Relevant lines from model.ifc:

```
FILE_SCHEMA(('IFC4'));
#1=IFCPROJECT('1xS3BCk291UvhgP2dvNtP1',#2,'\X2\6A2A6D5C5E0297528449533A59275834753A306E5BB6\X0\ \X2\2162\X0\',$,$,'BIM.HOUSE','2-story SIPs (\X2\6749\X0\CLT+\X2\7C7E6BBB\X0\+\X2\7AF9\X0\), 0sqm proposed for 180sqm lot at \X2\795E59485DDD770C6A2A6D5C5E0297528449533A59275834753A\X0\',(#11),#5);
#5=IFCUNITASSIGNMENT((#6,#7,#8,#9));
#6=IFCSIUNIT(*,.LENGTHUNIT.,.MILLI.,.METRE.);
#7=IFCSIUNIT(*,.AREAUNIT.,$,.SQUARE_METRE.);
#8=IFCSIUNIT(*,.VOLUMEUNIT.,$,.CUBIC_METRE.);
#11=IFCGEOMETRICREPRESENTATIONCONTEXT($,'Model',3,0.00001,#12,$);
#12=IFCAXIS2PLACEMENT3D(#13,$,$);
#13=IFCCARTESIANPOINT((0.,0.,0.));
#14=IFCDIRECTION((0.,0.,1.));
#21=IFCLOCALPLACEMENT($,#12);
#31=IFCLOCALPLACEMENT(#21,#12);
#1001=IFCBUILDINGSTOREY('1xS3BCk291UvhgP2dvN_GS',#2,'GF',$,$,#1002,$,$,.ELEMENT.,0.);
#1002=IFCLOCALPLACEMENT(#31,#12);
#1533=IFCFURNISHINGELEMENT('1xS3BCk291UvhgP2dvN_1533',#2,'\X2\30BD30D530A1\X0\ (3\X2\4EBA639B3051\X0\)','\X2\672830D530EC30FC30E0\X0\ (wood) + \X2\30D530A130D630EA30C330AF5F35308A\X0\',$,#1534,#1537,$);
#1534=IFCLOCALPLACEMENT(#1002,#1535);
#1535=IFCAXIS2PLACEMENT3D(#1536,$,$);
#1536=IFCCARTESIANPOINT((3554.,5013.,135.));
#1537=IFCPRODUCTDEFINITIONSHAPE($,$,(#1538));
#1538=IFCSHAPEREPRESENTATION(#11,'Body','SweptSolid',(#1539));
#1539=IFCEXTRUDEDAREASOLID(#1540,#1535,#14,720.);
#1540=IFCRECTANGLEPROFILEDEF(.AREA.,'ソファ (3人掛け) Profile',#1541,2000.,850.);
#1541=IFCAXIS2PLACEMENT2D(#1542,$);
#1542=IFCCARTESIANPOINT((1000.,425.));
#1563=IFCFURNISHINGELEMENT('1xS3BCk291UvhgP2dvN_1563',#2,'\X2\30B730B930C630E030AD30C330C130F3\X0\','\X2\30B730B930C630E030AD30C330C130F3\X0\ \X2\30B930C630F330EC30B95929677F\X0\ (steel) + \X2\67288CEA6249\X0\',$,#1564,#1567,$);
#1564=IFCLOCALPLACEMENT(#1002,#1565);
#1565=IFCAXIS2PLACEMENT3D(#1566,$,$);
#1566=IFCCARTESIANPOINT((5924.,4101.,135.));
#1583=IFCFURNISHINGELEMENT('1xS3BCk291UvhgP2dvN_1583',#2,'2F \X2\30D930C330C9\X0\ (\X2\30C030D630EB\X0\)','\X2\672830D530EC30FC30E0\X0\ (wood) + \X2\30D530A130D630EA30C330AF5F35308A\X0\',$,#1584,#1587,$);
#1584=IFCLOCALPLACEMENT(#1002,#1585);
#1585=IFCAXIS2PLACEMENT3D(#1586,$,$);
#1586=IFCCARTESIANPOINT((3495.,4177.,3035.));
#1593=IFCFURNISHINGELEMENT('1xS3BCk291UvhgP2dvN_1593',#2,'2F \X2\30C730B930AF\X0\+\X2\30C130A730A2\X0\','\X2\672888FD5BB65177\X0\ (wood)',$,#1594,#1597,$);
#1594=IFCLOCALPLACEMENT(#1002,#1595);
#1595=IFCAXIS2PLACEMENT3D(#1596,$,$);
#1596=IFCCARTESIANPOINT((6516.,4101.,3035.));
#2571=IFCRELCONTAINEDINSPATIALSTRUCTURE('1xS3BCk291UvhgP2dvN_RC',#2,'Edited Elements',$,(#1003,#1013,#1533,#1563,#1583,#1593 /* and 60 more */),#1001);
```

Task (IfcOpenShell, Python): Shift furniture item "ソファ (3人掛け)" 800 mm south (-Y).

```python
import ifcopenshell
import ifcopenshell.api.geometry
import ifcopenshell.util.placement

model = ifcopenshell.open("model.ifc")

item = model.by_guid("1xS3BCk291UvhgP2dvN_1533")
matrix = ifcopenshell.util.placement.get_local_placement(item.ObjectPlacement)
matrix[1, 3] -= 800.0
ifcopenshell.api.geometry.edit_object_placement(model, product=item, matrix=matrix, is_si=False)

print(ifcopenshell.util.placement.get_local_placement(item.ObjectPlacement).round(3) + 0.0)

model.write("model_edited.ifc")
```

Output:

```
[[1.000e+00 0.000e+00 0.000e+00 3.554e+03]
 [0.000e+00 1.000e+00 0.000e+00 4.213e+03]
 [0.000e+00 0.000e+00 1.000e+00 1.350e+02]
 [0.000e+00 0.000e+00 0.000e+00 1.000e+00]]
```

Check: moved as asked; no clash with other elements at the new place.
